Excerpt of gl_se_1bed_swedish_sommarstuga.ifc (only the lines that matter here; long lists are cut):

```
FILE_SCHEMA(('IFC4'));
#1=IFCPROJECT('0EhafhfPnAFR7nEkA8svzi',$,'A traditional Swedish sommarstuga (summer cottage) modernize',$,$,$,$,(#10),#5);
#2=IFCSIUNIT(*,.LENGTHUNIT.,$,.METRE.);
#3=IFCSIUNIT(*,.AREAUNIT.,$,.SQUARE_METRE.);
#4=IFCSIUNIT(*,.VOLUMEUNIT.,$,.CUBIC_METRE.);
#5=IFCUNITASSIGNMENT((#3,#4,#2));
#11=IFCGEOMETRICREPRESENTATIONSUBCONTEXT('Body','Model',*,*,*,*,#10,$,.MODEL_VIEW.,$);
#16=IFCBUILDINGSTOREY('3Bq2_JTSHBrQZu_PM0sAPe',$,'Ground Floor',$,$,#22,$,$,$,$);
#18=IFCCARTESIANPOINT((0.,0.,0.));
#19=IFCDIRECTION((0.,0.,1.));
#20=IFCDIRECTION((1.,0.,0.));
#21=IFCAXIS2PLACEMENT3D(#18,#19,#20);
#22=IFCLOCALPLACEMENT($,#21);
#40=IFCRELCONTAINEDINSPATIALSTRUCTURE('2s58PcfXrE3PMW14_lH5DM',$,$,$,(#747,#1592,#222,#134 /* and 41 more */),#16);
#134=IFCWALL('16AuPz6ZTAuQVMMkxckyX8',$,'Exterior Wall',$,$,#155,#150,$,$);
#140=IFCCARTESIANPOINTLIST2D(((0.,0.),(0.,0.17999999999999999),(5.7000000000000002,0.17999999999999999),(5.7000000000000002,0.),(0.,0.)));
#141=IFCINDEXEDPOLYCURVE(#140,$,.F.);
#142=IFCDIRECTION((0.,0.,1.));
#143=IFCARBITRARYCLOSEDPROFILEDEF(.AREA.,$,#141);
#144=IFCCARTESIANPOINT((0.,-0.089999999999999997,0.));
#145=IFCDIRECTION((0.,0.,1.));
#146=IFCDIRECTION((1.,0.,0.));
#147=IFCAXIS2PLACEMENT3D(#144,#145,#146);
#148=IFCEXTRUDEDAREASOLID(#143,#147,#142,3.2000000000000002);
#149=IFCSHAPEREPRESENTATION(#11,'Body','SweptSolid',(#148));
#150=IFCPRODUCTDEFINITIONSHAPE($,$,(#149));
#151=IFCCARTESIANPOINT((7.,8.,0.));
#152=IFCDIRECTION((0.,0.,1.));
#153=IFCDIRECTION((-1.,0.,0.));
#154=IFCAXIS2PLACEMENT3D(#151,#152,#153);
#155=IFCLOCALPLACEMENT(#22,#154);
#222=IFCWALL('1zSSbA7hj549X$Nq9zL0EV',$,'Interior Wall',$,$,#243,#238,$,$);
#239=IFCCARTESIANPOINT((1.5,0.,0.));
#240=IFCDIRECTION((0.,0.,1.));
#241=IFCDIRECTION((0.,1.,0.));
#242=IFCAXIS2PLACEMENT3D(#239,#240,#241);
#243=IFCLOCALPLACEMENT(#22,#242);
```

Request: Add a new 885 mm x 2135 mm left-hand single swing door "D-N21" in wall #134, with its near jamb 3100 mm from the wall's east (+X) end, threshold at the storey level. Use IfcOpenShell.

```python
import numpy as np
import ifcopenshell
import ifcopenshell.api.feature
import ifcopenshell.api.geometry
import ifcopenshell.api.root
import ifcopenshell.api.spatial
import ifcopenshell.geom
import ifcopenshell.util.element
import ifcopenshell.util.placement
import ifcopenshell.util.representation
import ifcopenshell.util.shape
import ifcopenshell.util.unit

model = ifcopenshell.open("gl_se_1bed_swedish_sommarstuga.ifc")
unit_scale = ifcopenshell.util.unit.calculate_unit_scale(model)
settings = ifcopenshell.geom.settings()


def volume(element):
    """Net volume in cubic metres, openings subtracted."""
    shape = ifcopenshell.geom.create_shape(settings, element)
    return ifcopenshell.util.shape.get_volume(shape.geometry)


wall = model.by_guid("16AuPz6ZTAuQVMMkxckyX8")
storey = ifcopenshell.util.element.get_container(wall, ifc_class="IfcBuildingStorey")
context = ifcopenshell.util.representation.get_context(model, "Model", "Body", "MODEL_VIEW")
before = volume(wall)

width, height, from_end, sill = 0.885, 2.135, 3.1, 0.0  # metres

# The wall runs along its own X axis, and the end named is its -X end.
wall_shape = ifcopenshell.geom.create_shape(settings, wall)
x, y, z = ifcopenshell.util.shape.get_vertices(wall_shape.geometry).T
start = x.min() + from_end
face, thickness = float(y.min()), float(y.max() - y.min())
wall_matrix = ifcopenshell.util.placement.get_local_placement(wall.ObjectPlacement)
level = ifcopenshell.util.placement.get_local_placement(storey.ObjectPlacement)[2, 3]


def in_wall(x, y):
    """Placement at x, y metres in the wall's axes, at sill height."""
    matrix = wall_matrix.copy()
    matrix[:, 3] = wall_matrix @ np.array([x / unit_scale, y / unit_scale, 0.0, 1.0])
    matrix[2, 3] = level + sill / unit_scale
    return matrix


# Opening: a box that overshoots both wall faces by 50 mm.
opening = ifcopenshell.api.root.create_entity(model, ifc_class="IfcOpeningElement", predefined_type="OPENING")
box = ifcopenshell.api.geometry.add_wall_representation(
    model, context=context, length=width, height=height, thickness=thickness + 0.1
)
ifcopenshell.api.geometry.assign_representation(model, product=opening, representation=box)
ifcopenshell.api.geometry.edit_object_placement(model, product=opening, matrix=in_wall(start, face - 0.05), is_si=False)
ifcopenshell.api.feature.add_feature(model, feature=opening, element=wall)

door = ifcopenshell.api.root.create_entity(model, ifc_class="IfcDoor", name="D-N21", predefined_type="DOOR")
door.OverallWidth, door.OverallHeight = width / unit_scale, height / unit_scale
door.OperationType = "SINGLE_SWING_LEFT"
body = ifcopenshell.api.geometry.add_door_representation(
    model,
    context=context,
    overall_width=door.OverallWidth,
    overall_height=door.OverallHeight,
    operation_type="SINGLE_SWING_LEFT",
    lining_properties={"LiningDepth": thickness / unit_scale, "ThresholdDepth": thickness / unit_scale},
)
ifcopenshell.api.geometry.assign_representation(model, product=door, representation=body)
ifcopenshell.api.spatial.assign_container(model, products=[door], relating_structure=storey)
ifcopenshell.api.feature.add_filling(model, opening=opening, element=door)

# The lining spans the wall, so the door starts at the wall face.
ifcopenshell.api.geometry.edit_object_placement(model, product=door, matrix=in_wall(start, face), is_si=False)

after = volume(wall)

print(f"wall volume {before:.3f} -> {after:.3f} m3")

model.write("gl_se_1bed_swedish_sommarstuga_v2.ifc")
```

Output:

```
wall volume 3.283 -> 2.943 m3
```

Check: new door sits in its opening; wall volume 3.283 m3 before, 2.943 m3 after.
